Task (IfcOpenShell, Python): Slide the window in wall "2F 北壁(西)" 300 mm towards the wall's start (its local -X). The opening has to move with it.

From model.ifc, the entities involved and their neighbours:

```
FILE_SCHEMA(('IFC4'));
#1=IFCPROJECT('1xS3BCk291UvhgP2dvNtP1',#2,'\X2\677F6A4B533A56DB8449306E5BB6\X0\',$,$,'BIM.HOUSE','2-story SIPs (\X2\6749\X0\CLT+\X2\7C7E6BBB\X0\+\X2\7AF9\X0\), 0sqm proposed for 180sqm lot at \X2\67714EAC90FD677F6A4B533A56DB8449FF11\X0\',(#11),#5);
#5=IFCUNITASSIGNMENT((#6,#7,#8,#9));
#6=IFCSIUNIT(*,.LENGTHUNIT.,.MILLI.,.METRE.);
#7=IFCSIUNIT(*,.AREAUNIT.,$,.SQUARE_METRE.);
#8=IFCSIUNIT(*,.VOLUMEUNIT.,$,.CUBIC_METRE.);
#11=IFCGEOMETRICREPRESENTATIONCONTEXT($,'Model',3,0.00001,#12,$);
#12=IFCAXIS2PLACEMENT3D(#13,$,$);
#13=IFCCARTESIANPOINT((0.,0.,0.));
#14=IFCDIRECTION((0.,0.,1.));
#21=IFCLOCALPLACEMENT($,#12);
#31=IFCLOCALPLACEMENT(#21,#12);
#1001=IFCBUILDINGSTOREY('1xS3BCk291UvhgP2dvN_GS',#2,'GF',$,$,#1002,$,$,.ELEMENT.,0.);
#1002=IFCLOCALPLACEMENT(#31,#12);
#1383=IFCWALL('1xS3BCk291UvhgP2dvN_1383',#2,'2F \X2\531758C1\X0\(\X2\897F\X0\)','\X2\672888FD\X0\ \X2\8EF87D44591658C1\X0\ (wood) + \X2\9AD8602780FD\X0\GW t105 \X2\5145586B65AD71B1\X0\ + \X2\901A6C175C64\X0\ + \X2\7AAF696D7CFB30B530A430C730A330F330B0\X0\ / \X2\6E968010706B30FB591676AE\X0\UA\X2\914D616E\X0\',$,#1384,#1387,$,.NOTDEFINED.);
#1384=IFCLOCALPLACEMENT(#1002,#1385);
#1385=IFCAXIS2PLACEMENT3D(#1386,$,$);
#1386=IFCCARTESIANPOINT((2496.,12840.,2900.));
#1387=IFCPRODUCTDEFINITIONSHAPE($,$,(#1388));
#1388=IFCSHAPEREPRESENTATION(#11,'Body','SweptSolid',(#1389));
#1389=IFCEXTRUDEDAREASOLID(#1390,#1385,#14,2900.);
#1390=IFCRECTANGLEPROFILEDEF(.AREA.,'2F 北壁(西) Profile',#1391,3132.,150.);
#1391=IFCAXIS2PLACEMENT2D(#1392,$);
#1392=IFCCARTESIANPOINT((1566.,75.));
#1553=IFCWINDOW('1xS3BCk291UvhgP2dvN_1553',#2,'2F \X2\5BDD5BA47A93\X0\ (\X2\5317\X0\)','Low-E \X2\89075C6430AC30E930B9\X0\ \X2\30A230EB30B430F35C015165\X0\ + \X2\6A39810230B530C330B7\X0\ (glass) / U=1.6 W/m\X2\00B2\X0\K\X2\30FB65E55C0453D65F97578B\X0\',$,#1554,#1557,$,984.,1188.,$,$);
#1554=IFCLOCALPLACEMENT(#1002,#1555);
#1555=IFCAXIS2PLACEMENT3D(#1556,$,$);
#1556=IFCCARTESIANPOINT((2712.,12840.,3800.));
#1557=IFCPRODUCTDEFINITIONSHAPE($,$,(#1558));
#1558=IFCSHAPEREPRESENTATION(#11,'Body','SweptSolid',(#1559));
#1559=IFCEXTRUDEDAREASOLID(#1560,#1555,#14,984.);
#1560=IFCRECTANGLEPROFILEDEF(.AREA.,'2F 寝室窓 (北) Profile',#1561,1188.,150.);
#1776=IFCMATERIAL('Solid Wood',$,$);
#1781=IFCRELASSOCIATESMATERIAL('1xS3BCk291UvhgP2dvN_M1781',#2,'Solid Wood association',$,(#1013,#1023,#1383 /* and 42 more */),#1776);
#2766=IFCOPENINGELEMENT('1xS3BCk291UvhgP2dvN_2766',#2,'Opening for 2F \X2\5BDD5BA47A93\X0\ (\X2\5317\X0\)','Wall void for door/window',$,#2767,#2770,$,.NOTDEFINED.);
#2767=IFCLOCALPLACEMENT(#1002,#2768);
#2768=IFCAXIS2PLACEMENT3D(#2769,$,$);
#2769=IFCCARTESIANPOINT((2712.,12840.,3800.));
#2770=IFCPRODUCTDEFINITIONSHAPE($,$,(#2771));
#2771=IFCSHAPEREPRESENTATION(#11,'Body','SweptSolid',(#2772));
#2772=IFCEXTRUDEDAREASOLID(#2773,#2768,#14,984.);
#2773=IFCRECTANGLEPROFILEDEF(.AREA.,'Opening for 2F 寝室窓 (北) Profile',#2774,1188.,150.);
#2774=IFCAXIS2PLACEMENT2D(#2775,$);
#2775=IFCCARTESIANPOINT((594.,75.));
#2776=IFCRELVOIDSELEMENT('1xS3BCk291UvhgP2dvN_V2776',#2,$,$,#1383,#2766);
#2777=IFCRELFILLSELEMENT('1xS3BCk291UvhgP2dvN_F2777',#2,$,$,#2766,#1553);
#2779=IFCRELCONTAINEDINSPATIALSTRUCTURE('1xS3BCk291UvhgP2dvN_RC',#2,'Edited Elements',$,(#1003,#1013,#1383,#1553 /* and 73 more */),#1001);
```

```python
import ifcopenshell
import ifcopenshell.api.geometry
import ifcopenshell.util.placement
import ifcopenshell.util.unit

model = ifcopenshell.open("model.ifc")
unit_scale = ifcopenshell.util.unit.calculate_unit_scale(model)

window = model.by_guid("1xS3BCk291UvhgP2dvN_1553")
opening = window.FillsVoids[0].RelatingOpeningElement
wall = opening.VoidsElements[0].RelatingBuildingElement

wall_matrix = ifcopenshell.util.placement.get_local_placement(wall.ObjectPlacement)
shift = wall_matrix[:3, 0] * -0.3 / unit_scale
before = ifcopenshell.util.placement.get_local_placement(window.ObjectPlacement)[:3, 3].copy()

# The window is not placed relative to its opening, so move both.
for product in (opening, window):
    matrix = ifcopenshell.util.placement.get_local_placement(product.ObjectPlacement)
    matrix[:3, 3] += shift
    ifcopenshell.api.geometry.edit_object_placement(model, product=product, matrix=matrix, is_si=False)

after = ifcopenshell.util.placement.get_local_placement(window.ObjectPlacement)[:3, 3]
print("window moved by", (after - before).round(3) + 0.0)

model.write("model_updated.ifc")
```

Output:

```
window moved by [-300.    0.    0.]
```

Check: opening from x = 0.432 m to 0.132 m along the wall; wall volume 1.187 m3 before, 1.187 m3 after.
